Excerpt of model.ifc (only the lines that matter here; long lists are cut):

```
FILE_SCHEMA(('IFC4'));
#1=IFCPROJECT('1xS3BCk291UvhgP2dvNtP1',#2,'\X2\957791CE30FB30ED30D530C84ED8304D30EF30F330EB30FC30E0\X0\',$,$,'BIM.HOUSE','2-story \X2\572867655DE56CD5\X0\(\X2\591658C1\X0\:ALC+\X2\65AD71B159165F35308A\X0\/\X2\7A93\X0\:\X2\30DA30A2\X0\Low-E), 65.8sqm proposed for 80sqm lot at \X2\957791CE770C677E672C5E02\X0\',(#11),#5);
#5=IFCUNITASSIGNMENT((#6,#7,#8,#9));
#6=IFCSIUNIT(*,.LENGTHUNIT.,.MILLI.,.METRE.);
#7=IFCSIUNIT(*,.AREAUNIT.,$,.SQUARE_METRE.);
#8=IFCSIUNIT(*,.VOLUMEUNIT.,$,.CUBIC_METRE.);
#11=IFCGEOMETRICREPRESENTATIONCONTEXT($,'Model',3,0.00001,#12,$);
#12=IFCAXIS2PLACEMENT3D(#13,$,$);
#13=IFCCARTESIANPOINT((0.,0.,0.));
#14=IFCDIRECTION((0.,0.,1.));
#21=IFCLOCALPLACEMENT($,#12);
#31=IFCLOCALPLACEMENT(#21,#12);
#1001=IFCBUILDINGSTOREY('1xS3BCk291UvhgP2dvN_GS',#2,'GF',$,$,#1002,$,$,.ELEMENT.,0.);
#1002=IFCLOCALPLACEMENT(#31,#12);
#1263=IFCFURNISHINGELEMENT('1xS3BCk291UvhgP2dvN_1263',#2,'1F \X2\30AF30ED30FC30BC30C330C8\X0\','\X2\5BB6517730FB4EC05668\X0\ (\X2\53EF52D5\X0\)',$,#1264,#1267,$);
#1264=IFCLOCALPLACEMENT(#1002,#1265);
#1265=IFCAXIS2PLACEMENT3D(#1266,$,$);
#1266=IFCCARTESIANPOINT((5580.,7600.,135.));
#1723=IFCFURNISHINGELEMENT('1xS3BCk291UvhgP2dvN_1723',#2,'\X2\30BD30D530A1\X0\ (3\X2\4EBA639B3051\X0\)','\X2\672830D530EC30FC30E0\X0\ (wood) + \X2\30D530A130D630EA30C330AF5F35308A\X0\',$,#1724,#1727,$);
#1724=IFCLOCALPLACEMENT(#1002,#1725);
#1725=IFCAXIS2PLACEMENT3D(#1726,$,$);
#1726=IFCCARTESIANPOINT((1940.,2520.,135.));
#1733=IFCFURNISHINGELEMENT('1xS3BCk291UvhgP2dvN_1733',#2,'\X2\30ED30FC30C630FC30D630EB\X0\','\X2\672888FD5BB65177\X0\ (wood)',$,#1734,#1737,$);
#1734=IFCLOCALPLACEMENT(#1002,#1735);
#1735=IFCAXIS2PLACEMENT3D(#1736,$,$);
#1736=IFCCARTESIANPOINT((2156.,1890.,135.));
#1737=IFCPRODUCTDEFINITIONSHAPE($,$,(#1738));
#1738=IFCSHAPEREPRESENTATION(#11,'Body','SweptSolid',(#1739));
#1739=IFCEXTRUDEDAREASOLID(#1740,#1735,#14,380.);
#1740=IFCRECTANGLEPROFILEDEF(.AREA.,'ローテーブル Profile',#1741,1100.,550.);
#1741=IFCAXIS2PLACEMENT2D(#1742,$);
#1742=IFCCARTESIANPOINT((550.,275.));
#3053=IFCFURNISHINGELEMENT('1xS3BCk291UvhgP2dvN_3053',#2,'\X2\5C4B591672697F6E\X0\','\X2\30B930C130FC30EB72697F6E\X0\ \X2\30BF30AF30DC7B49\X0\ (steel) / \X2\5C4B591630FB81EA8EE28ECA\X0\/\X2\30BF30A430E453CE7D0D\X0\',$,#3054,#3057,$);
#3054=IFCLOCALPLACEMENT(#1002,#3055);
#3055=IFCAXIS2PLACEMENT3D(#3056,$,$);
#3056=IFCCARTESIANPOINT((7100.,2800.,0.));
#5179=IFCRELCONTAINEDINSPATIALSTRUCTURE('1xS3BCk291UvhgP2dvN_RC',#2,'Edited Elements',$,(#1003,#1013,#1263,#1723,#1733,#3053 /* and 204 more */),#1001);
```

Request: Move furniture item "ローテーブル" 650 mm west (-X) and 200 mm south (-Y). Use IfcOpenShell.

```python
import ifcopenshell
import ifcopenshell.api.geometry
import ifcopenshell.util.placement

model = ifcopenshell.open("model.ifc")

item = model.by_id(1733)
matrix = ifcopenshell.util.placement.get_local_placement(item.ObjectPlacement)
matrix[0, 3] -= 650.0
matrix[1, 3] -= 200.0
ifcopenshell.api.geometry.edit_object_placement(model, product=item, matrix=matrix, is_si=False)

print(ifcopenshell.util.placement.get_local_placement(item.ObjectPlacement).round(3) + 0.0)

model.write("model_rev.ifc")
```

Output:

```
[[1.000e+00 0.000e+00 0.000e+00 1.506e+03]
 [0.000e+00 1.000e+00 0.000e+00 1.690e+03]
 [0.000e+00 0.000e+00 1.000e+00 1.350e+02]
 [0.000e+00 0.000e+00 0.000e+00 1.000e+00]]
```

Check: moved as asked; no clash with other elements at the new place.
